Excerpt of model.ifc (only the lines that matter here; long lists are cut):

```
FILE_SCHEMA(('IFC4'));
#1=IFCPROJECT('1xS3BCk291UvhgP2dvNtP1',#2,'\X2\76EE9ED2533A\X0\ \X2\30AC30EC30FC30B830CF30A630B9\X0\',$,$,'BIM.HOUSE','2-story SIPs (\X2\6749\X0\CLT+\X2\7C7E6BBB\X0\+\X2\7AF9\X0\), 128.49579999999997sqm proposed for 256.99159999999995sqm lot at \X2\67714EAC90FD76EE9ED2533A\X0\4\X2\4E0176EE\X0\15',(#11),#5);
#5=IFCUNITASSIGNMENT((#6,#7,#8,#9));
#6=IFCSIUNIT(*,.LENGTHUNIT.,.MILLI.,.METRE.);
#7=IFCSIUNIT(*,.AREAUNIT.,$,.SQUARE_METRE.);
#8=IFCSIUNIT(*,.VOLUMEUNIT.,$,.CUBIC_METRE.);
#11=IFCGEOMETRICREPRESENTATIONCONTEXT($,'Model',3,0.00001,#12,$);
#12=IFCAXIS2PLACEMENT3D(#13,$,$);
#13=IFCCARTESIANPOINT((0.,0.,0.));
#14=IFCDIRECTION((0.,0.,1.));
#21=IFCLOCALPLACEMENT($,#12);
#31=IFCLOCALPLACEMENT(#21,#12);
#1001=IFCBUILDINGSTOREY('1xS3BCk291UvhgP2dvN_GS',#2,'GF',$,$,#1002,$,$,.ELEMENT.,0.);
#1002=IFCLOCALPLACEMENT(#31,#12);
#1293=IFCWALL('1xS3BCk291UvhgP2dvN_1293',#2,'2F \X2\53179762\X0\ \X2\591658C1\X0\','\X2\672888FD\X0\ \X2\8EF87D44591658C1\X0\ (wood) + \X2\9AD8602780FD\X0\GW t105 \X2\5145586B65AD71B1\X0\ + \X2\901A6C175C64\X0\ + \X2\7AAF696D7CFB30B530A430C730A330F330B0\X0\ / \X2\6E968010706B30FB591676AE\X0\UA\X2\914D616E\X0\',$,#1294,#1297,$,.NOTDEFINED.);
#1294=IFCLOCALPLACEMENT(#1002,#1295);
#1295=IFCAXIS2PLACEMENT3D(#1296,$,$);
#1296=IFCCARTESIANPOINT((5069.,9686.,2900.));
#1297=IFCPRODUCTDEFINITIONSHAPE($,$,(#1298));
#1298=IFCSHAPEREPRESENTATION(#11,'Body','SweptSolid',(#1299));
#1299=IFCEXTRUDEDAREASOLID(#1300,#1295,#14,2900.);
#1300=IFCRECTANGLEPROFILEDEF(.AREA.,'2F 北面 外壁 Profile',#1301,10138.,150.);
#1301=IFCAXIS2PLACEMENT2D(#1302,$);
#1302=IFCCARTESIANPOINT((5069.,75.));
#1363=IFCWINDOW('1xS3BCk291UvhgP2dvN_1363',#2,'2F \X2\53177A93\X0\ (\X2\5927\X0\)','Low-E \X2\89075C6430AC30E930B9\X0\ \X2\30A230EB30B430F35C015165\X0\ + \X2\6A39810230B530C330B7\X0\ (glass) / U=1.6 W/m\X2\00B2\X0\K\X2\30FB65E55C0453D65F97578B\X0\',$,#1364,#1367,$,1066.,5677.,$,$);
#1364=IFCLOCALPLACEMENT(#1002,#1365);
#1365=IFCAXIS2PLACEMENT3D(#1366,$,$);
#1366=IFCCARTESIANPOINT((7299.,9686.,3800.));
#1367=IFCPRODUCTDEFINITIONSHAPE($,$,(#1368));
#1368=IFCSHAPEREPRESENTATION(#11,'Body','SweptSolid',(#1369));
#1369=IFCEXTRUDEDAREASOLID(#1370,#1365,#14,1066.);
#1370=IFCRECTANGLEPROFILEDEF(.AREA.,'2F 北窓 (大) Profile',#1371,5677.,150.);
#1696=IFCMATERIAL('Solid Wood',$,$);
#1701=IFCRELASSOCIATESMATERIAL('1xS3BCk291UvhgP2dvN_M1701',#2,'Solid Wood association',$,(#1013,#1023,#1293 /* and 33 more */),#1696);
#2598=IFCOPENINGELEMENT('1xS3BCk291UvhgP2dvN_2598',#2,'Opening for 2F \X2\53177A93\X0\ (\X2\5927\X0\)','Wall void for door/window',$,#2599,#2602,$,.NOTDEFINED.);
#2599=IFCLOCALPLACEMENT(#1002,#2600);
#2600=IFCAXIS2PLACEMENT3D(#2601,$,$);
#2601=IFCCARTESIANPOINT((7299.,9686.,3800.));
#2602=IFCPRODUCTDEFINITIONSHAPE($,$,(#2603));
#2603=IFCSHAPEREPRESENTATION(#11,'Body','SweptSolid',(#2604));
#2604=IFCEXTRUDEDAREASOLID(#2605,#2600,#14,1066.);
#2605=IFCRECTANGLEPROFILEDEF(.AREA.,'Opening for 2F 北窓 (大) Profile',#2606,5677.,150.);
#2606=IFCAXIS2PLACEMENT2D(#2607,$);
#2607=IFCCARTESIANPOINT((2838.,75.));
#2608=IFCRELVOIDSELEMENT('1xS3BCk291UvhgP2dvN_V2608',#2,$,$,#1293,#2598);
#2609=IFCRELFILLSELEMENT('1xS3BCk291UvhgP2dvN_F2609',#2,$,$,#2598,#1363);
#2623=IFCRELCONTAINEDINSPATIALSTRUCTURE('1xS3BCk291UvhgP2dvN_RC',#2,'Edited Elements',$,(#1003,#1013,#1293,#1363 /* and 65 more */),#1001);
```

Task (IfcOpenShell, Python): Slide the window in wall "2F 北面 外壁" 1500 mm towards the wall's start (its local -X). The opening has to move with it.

```python
import ifcopenshell
import ifcopenshell.api.geometry
import ifcopenshell.util.placement
import ifcopenshell.util.unit

model = ifcopenshell.open("model.ifc")
unit_scale = ifcopenshell.util.unit.calculate_unit_scale(model)

window = model.by_id(1363)
opening = window.FillsVoids[0].RelatingOpeningElement
wall = opening.VoidsElements[0].RelatingBuildingElement

wall_matrix = ifcopenshell.util.placement.get_local_placement(wall.ObjectPlacement)
shift = wall_matrix[:3, 0] * -1.5 / unit_scale
before = ifcopenshell.util.placement.get_local_placement(window.ObjectPlacement)[:3, 3].copy()

# The window is not placed relative to its opening, so move both.
for product in (opening, window):
    matrix = ifcopenshell.util.placement.get_local_placement(product.ObjectPlacement)
    matrix[:3, 3] += shift
    ifcopenshell.api.geometry.edit_object_placement(model, product=product, matrix=matrix, is_si=False)

after = ifcopenshell.util.placement.get_local_placement(window.ObjectPlacement)[:3, 3]
print("window moved by", (after - before).round(3) + 0.0)

model.write("model_rev.ifc")
```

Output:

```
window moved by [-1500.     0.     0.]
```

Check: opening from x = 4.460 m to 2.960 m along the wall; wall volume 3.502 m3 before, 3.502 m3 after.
